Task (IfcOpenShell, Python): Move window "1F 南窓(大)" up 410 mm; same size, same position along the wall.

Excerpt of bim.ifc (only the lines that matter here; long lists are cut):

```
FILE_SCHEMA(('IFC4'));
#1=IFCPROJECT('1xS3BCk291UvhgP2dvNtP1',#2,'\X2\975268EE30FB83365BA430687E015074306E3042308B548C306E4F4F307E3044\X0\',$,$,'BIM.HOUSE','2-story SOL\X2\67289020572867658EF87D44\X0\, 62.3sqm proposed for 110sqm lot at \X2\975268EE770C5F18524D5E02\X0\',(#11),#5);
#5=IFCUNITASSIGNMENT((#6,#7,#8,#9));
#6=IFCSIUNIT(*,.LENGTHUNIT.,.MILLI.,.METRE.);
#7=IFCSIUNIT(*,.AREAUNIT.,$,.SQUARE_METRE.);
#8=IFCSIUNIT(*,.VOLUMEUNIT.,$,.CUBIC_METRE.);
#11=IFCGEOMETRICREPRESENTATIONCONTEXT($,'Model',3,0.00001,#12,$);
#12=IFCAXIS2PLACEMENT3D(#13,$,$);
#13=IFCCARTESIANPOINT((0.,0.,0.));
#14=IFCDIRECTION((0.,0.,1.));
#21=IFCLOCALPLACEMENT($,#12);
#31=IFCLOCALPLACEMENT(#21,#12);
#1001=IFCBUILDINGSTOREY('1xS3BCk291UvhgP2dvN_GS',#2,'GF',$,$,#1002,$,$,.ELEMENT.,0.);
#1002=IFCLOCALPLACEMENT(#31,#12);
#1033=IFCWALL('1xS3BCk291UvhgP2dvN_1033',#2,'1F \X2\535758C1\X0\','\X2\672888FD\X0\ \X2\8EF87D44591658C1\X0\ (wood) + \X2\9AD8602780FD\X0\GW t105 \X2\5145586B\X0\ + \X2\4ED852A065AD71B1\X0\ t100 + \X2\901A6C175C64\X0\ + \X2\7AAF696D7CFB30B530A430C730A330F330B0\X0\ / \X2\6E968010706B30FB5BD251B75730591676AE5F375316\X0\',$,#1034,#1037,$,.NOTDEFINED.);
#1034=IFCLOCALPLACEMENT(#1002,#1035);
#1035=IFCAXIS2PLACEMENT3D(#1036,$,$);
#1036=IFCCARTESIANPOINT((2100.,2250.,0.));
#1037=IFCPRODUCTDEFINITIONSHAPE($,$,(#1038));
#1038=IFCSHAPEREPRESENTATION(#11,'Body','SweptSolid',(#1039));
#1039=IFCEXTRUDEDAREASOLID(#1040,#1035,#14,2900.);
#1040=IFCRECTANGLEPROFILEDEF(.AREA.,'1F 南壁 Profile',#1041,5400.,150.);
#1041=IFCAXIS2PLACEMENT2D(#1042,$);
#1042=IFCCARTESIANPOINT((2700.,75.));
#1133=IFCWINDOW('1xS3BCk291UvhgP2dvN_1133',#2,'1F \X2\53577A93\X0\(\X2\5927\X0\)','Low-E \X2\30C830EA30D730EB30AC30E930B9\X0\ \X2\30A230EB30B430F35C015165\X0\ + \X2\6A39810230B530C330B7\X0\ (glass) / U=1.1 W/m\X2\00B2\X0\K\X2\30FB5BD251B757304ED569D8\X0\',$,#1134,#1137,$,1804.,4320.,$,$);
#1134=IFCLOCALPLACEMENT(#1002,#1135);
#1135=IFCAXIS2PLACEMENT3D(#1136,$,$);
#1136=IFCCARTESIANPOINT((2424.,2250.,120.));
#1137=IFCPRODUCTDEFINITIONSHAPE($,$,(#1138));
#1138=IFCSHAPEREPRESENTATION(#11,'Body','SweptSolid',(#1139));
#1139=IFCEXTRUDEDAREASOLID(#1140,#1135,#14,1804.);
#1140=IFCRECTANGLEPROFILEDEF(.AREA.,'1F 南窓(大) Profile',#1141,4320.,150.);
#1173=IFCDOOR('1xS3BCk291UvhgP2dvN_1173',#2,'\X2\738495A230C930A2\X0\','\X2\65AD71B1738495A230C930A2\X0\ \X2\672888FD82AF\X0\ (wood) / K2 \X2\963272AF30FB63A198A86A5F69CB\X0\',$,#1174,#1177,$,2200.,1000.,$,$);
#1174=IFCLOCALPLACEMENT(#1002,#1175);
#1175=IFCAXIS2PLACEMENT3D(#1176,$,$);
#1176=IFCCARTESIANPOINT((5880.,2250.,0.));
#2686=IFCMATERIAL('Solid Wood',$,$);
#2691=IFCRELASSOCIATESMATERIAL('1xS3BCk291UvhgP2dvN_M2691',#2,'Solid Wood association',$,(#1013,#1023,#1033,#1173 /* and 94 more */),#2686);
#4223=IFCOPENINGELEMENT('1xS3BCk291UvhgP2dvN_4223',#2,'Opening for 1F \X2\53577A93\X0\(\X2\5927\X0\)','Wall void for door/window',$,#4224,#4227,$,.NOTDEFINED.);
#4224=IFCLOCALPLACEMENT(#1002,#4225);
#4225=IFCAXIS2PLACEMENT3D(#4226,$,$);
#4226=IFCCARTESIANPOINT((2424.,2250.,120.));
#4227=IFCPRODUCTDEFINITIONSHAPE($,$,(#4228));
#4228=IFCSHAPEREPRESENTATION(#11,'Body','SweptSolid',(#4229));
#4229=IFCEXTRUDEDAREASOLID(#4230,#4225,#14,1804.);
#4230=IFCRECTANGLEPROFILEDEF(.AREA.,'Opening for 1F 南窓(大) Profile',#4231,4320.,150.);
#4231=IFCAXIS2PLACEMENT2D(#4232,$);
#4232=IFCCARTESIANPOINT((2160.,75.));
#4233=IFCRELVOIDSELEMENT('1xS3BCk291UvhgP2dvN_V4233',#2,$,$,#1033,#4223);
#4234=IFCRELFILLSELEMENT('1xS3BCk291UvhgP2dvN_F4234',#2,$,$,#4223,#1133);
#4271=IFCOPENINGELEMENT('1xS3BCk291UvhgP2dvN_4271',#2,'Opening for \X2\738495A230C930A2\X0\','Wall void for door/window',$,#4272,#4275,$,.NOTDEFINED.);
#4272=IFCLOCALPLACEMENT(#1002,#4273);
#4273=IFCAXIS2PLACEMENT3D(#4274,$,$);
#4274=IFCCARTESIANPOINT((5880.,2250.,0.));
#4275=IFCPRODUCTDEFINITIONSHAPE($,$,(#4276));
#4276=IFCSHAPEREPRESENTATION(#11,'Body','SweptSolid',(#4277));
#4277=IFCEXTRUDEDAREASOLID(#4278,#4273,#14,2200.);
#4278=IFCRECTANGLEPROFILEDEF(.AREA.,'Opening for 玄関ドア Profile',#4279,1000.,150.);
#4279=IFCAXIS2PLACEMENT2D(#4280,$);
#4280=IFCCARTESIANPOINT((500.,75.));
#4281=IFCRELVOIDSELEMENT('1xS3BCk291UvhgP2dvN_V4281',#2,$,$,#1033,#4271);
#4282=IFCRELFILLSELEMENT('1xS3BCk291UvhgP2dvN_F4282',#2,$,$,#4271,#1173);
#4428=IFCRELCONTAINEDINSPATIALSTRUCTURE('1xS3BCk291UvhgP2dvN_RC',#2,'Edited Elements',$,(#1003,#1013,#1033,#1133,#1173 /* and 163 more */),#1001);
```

```python
import numpy as np
import ifcopenshell
import ifcopenshell.api.geometry
import ifcopenshell.util.placement
import ifcopenshell.util.unit

model = ifcopenshell.open("bim.ifc")
unit_scale = ifcopenshell.util.unit.calculate_unit_scale(model)

window = model.by_id(1133)
opening = window.FillsVoids[0].RelatingOpeningElement
dz = 0.41 / unit_scale

shift = np.array([0.0, 0.0, dz])
# The window is not placed relative to its opening, so move both.
for product in (opening, window):
    matrix = ifcopenshell.util.placement.get_local_placement(product.ObjectPlacement)
    matrix[:3, 3] += shift
    ifcopenshell.api.geometry.edit_object_placement(model, product=product, matrix=matrix, is_si=False)

print(f"moved by {dz * unit_scale:+.3f} m")

model.write("bim_v2.ifc")
```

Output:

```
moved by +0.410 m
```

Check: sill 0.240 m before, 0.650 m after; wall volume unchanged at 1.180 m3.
